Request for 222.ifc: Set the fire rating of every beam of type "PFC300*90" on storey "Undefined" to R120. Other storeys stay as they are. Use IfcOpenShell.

First a look at what the model holds.

```python
import ifcopenshell
import ifcopenshell.util.element

model = ifcopenshell.open("222.ifc")
print(model.schema)
storey = next(s for s in model.by_type("IfcBuildingStorey") if s.Name == "Undefined")
beams = [e for e in ifcopenshell.util.element.get_decomposition(storey) if e.is_a("IfcBeam")]
seen = {}
for e in beams:
    element_type = ifcopenshell.util.element.get_type(e)
    key = (element_type.Name if element_type != e and element_type else None, ifcopenshell.util.element.get_pset(e, "Pset_BeamCommon", "FireRating"))
    seen[key] = seen.get(key, 0) + 1
for (name, value), count in sorted(seen.items(), key=str):
    print(count, "x", name, "|", value)
```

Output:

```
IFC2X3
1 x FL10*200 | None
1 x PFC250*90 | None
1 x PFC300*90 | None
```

```python
import ifcopenshell
import ifcopenshell.api.pset
import ifcopenshell.util.element

model = ifcopenshell.open("222.ifc")

storey = next(s for s in model.by_type("IfcBuildingStorey") if s.Name == "Undefined")
beams = [e for e in ifcopenshell.util.element.get_decomposition(storey) if e.is_a("IfcBeam")]

count = 0
for e in beams:
    element_type = ifcopenshell.util.element.get_type(e)
    if element_type in (None, e) or element_type.Name != "PFC300*90":
        continue
    # add_pset returns the element's existing set when there is one.
    pset = ifcopenshell.api.pset.add_pset(model, product=e, name="Pset_BeamCommon")
    ifcopenshell.api.pset.edit_pset(model, pset=pset, properties={"FireRating": "R120"})
    count += 1

print(count, "beams updated")

model.write("222_v2.ifc")
```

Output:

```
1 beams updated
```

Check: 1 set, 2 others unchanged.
